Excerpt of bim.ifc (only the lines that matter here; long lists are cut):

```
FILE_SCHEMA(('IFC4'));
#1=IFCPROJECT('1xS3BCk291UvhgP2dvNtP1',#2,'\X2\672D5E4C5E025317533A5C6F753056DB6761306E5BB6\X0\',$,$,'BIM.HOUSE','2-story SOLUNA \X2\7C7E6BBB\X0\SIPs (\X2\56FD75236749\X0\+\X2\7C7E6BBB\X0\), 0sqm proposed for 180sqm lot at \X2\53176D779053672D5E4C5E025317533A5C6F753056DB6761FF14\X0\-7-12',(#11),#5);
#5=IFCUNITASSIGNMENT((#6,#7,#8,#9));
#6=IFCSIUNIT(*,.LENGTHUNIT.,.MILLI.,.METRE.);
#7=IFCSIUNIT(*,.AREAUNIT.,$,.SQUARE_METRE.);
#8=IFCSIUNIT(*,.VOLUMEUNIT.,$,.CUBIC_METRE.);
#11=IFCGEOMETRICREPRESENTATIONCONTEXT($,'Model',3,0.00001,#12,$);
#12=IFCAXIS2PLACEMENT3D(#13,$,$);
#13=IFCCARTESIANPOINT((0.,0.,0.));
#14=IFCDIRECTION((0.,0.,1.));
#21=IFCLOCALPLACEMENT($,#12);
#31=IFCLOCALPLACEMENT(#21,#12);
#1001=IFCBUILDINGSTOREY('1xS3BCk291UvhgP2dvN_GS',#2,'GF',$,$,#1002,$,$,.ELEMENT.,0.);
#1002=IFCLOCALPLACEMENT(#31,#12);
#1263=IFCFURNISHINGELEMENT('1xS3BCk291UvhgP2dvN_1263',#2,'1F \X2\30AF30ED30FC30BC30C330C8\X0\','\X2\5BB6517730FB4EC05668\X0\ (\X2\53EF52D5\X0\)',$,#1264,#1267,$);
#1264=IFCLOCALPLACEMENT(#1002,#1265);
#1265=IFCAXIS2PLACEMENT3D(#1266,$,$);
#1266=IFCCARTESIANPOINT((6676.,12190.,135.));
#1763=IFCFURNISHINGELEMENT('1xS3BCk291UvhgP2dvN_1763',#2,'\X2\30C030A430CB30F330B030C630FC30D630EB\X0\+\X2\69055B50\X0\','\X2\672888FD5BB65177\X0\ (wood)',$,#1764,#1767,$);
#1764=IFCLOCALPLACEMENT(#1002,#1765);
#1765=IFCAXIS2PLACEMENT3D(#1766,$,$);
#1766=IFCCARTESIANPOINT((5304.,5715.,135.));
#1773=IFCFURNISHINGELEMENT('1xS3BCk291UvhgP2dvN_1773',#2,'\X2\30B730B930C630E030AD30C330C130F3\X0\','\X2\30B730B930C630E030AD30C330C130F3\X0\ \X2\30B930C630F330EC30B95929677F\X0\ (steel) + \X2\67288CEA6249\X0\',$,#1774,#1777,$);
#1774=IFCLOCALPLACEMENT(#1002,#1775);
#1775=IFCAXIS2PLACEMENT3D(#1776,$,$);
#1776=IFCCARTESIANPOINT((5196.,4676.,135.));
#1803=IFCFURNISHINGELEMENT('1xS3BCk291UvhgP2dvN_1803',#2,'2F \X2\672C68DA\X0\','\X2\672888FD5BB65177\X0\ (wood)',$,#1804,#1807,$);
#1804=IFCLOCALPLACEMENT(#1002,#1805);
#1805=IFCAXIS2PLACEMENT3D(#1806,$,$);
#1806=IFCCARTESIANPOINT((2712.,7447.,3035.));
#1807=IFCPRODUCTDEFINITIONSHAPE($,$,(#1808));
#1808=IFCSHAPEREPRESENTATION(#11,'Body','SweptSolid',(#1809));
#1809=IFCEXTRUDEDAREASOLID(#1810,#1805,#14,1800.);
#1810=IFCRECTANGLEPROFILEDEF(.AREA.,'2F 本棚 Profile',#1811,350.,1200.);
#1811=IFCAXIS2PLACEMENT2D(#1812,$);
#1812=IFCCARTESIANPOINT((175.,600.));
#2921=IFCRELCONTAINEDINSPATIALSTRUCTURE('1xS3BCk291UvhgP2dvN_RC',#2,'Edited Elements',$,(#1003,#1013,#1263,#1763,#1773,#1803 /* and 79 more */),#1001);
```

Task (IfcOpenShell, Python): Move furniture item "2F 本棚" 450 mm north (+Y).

```python
import ifcopenshell
import ifcopenshell.api.geometry
import ifcopenshell.util.placement
import ifcopenshell.util.unit

model = ifcopenshell.open("bim.ifc")
unit_scale = ifcopenshell.util.unit.calculate_unit_scale(model)

item = model.by_guid("1xS3BCk291UvhgP2dvN_1803")
matrix = ifcopenshell.util.placement.get_local_placement(item.ObjectPlacement)
matrix[1, 3] += 0.45 / unit_scale
ifcopenshell.api.geometry.edit_object_placement(model, product=item, matrix=matrix, is_si=False)

print(ifcopenshell.util.placement.get_local_placement(item.ObjectPlacement).round(3) + 0.0)

model.write("bim_edited.ifc")
```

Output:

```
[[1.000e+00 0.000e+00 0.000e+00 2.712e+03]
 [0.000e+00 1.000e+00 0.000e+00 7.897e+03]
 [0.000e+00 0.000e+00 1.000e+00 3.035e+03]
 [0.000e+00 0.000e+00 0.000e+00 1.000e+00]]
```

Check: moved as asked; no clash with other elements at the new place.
